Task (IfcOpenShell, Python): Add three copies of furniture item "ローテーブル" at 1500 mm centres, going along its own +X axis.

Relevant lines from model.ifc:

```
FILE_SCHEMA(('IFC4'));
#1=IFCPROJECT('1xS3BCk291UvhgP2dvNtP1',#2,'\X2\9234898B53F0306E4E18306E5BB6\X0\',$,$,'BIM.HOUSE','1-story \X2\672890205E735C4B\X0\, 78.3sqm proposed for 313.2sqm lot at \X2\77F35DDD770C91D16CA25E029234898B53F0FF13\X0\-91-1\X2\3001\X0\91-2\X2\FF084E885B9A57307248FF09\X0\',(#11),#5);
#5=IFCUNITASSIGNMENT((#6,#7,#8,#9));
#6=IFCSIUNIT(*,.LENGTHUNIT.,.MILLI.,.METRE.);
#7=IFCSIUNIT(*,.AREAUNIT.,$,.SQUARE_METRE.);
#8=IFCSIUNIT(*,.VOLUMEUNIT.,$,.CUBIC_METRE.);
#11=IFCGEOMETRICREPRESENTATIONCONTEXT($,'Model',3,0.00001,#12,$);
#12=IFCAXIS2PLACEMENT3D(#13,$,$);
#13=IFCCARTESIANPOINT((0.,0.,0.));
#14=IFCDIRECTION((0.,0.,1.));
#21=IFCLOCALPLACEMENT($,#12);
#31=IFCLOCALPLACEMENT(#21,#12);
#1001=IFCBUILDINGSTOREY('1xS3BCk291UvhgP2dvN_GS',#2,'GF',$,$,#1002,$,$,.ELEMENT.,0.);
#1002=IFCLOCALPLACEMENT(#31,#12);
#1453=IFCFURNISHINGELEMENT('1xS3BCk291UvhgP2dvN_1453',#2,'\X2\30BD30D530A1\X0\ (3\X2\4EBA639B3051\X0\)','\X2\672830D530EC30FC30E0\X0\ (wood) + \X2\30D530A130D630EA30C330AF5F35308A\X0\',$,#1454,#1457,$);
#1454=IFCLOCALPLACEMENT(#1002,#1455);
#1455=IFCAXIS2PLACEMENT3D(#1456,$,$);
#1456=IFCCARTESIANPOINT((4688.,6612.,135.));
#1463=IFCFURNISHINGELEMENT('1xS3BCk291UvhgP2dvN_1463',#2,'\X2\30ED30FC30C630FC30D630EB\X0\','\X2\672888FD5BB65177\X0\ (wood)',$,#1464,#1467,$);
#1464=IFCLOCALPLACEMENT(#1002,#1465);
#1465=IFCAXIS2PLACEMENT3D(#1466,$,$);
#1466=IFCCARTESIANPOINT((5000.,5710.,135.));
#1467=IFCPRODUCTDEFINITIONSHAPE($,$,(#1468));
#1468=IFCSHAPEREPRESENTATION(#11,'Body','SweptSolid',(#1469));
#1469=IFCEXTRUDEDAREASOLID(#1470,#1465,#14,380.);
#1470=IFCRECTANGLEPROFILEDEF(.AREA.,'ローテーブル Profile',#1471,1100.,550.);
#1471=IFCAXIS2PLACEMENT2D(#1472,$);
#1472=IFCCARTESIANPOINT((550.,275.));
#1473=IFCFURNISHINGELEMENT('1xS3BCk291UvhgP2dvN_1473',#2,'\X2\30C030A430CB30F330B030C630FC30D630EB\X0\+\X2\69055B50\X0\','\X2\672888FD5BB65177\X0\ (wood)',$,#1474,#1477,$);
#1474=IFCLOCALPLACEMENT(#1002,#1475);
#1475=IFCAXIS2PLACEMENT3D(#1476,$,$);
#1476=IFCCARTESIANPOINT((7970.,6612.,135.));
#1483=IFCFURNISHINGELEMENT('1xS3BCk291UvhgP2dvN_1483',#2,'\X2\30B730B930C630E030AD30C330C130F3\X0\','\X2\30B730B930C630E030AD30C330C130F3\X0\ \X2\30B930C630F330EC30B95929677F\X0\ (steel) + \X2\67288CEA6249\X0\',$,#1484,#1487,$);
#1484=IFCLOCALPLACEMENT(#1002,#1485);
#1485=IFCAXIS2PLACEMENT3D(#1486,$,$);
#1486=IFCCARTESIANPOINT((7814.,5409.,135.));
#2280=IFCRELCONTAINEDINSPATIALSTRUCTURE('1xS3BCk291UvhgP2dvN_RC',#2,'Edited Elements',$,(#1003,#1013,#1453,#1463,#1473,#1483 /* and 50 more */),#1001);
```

```python
import ifcopenshell
import ifcopenshell.api.geometry
import ifcopenshell.api.root
import ifcopenshell.util.element
import ifcopenshell.util.placement

model = ifcopenshell.open("model.ifc")


def reuse_history(source, copy):
    """copy_class also copies each property set's owner history, people and application; keep the originals."""
    for rel in copy.IsDefinedBy:
        if rel.is_a("IfcRelDefinesByProperties") and (history := rel.RelatingPropertyDefinition.OwnerHistory):
            rel.RelatingPropertyDefinition.OwnerHistory = source.OwnerHistory
            ifcopenshell.util.element.remove_deep2(model, history)


source = model.by_id(1463)
base = ifcopenshell.util.placement.get_local_placement(source.ObjectPlacement)
step = base[:3, 0] * 1500.0

for i in range(1, 4):
    copy = ifcopenshell.api.root.copy_class(model, product=source)
    copy.Representation = ifcopenshell.util.element.copy_deep(
        model, source.Representation, exclude=["IfcGeometricRepresentationContext", "IfcRepresentationMap"]
    )
    reuse_history(source, copy)
    matrix = base.copy()
    matrix[:3, 3] += i * step
    print("added at", matrix[:3, 3].round(3) + 0.0)
    ifcopenshell.api.geometry.edit_object_placement(model, product=copy, matrix=matrix, is_si=False)

model.write("model_v2.ifc")
```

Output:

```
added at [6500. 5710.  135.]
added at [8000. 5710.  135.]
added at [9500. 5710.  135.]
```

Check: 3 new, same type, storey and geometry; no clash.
